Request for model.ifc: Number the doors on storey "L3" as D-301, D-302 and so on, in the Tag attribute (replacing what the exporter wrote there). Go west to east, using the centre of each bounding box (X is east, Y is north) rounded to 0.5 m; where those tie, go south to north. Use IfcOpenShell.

First a look at what the model holds.

```python
import ifcopenshell
import ifcopenshell.util.element
import ifcopenshell.util.placement

model = ifcopenshell.open("model.ifc")
print(model.schema)
storey = next(s for s in model.by_type("IfcBuildingStorey") if s.Name == "L3")
doors = [e for e in ifcopenshell.util.element.get_decomposition(storey) if e.is_a("IfcDoor")]
for e in sorted(doors, key=lambda e: e.id()):
    origin = ifcopenshell.util.placement.get_local_placement(e.ObjectPlacement)[:3, 3]
    print(e.id(), e.Tag, e.Name, origin.round(2) + 0.0, sep=" | ")
```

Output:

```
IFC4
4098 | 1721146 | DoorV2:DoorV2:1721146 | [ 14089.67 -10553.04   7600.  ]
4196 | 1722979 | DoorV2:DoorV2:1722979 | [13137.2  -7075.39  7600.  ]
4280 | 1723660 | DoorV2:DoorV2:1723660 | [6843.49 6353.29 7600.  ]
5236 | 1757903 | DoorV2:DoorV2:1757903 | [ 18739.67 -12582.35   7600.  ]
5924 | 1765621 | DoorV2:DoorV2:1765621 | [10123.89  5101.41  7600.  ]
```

```python
import ifcopenshell
import ifcopenshell.geom
import ifcopenshell.util.element
import ifcopenshell.util.shape

model = ifcopenshell.open("model.ifc")
settings = ifcopenshell.geom.settings()
settings.set("use-world-coords", True)


def centre(element):
    shape = ifcopenshell.geom.create_shape(settings, element)
    return ifcopenshell.util.shape.get_bbox_centroid(shape.geometry)


storey = next(s for s in model.by_type("IfcBuildingStorey") if s.Name == "L3")
doors = [e for e in ifcopenshell.util.element.get_decomposition(storey) if e.is_a("IfcDoor")]

# Insertion points can sit at a corner or the storey origin, so sort by the geometry (in metres).
centres = {e: centre(e) for e in doors}
doors.sort(key=lambda e: (round(centres[e][0] / 0.5), centres[e][1]))

for i, e in enumerate(doors, start=1):
    number = f"D-3{i:02d}"
    e.Tag = number
    print(e.id(), number)

model.write("model_edited.ifc")
```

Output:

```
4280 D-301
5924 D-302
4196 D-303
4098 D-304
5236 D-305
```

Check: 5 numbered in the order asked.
